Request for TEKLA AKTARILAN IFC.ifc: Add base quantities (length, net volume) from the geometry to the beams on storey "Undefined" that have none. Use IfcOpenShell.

First a look at what the model holds.

```python
import ifcopenshell
import ifcopenshell.util.element
import ifcopenshell.util.unit

model = ifcopenshell.open("TEKLA AKTARILAN IFC.ifc")
print(model.schema)
for unit_type in ("LENGTHUNIT", "AREAUNIT", "VOLUMEUNIT"):
    print(unit_type, ifcopenshell.util.unit.calculate_unit_scale(model, unit_type))
storey = next(s for s in model.by_type("IfcBuildingStorey") if s.Name == "Undefined")
beams = [e for e in ifcopenshell.util.element.get_decomposition(storey) if e.is_a("IfcBeam")]
for e in sorted(beams, key=lambda e: e.id()):
    print(e.id(), e.is_a(), e.Name, list(ifcopenshell.util.element.get_psets(e, qtos_only=True)), sep=" | ")
```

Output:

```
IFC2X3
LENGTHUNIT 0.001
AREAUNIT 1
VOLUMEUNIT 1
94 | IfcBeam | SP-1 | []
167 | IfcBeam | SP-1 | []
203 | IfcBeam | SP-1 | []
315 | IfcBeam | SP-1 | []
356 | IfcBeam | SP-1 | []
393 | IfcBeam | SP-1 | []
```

```python
import ifcopenshell
import ifcopenshell.api.pset
import ifcopenshell.geom
import ifcopenshell.util.element
import ifcopenshell.util.shape
import ifcopenshell.util.unit

model = ifcopenshell.open("TEKLA AKTARILAN IFC.ifc")
unit_scale = ifcopenshell.util.unit.calculate_unit_scale(model)
volume_scale = ifcopenshell.util.unit.calculate_unit_scale(model, "VOLUMEUNIT")
settings = ifcopenshell.geom.settings()

storey = next(s for s in model.by_type("IfcBuildingStorey") if s.Name == "Undefined")
beams = [e for e in ifcopenshell.util.element.get_decomposition(storey) if e.is_a("IfcBeam")]

for e in sorted(beams, key=lambda e: e.id()):
    if ifcopenshell.util.element.get_psets(e, qtos_only=True, should_inherit=False):
        continue
    # Geometry comes back in metres, in the element's own axes.
    shape = ifcopenshell.geom.create_shape(settings, e)
    values = {
        "Length": ifcopenshell.util.shape.get_max_xyz(shape.geometry) / unit_scale,
        "NetVolume": ifcopenshell.util.shape.get_volume(shape.geometry) / volume_scale,
    }
    qto = ifcopenshell.api.pset.add_qto(model, product=e, name="BaseQuantities")
    ifcopenshell.api.pset.edit_qto(model, qto=qto, properties=values)
    print(e.id(), {k: round(v, 3) for k, v in values.items()})

model.write("TEKLA AKTARILAN IFC-out.ifc")
```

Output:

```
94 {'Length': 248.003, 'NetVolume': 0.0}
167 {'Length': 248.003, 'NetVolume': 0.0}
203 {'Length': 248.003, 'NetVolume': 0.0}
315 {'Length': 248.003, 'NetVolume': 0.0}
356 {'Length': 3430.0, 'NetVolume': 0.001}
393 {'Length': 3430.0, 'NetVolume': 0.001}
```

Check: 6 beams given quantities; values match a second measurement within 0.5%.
